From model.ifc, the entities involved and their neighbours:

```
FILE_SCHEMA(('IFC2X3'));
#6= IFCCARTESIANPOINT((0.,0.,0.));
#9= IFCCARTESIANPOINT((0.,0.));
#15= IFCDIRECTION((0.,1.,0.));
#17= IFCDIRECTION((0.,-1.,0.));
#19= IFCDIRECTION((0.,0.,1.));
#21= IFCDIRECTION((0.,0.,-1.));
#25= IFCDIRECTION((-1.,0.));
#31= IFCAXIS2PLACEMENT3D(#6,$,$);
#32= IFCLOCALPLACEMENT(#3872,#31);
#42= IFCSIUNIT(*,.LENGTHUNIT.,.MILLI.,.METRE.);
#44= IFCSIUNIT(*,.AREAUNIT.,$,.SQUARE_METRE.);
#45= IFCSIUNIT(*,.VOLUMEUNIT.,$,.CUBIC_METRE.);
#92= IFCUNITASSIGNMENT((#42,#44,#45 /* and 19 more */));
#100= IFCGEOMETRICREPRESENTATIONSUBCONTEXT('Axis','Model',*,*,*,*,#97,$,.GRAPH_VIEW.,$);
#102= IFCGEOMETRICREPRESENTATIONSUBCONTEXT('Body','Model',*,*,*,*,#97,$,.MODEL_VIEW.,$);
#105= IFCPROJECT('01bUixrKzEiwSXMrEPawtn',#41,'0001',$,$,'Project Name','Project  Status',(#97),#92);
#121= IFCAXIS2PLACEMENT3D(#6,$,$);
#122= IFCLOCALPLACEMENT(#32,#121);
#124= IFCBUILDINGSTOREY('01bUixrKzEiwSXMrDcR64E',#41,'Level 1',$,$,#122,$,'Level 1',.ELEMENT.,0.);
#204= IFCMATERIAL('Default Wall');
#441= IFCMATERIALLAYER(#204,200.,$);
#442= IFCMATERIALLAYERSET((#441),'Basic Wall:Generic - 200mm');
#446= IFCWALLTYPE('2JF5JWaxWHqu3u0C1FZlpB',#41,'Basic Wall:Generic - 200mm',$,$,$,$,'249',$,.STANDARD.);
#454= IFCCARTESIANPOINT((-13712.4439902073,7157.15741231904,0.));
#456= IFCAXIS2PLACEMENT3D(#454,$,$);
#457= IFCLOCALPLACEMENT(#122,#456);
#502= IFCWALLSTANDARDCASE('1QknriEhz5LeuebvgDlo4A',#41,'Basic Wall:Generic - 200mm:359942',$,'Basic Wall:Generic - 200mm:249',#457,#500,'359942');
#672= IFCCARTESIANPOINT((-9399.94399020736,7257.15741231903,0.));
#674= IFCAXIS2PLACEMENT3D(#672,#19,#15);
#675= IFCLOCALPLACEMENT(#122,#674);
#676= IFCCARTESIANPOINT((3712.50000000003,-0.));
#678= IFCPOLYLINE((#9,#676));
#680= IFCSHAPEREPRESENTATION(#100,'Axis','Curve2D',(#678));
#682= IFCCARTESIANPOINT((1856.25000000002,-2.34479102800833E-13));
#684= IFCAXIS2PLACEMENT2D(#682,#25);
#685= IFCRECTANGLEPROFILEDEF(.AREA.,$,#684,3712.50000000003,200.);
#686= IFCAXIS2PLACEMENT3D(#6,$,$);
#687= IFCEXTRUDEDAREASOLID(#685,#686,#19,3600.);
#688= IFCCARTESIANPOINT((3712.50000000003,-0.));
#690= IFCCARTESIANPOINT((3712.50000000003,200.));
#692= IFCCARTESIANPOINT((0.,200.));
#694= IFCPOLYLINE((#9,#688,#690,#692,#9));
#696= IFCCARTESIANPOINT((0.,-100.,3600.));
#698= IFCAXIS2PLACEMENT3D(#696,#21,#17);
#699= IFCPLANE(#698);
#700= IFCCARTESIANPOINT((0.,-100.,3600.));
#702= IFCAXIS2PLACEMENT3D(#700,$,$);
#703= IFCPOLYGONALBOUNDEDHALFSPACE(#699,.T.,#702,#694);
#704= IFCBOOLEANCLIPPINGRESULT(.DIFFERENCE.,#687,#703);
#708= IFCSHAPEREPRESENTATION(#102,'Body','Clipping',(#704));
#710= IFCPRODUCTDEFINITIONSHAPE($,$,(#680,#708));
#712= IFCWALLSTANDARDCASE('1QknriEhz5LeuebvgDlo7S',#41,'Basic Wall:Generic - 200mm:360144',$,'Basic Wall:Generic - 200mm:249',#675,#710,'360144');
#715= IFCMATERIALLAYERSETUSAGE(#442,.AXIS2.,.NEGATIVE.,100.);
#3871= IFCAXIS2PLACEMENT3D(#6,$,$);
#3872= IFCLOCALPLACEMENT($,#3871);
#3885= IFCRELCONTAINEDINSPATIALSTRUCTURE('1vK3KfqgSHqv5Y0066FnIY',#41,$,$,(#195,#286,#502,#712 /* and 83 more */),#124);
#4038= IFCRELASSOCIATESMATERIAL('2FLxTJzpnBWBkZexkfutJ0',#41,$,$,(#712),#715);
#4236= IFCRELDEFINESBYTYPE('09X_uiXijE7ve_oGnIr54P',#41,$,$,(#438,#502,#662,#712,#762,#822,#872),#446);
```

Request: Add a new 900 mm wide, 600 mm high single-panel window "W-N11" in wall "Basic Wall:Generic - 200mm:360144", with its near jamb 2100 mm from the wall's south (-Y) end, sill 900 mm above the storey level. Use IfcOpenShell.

```python
import numpy as np
import ifcopenshell
import ifcopenshell.api.feature
import ifcopenshell.api.geometry
import ifcopenshell.api.root
import ifcopenshell.api.spatial
import ifcopenshell.api.type
import ifcopenshell.geom
import ifcopenshell.util.element
import ifcopenshell.util.placement
import ifcopenshell.util.representation
import ifcopenshell.util.shape
import ifcopenshell.util.unit

model = ifcopenshell.open("model.ifc")
unit_scale = ifcopenshell.util.unit.calculate_unit_scale(model)
settings = ifcopenshell.geom.settings()


def volume(element):
    """Net volume in cubic metres, openings subtracted."""
    shape = ifcopenshell.geom.create_shape(settings, element)
    return ifcopenshell.util.shape.get_volume(shape.geometry)


wall = model.by_guid("1QknriEhz5LeuebvgDlo7S")
storey = ifcopenshell.util.element.get_container(wall, ifc_class="IfcBuildingStorey")
context = ifcopenshell.util.representation.get_context(model, "Model", "Body", "MODEL_VIEW")
before = volume(wall)

width, height, from_end, sill = 0.9, 0.6, 2.1, 0.9  # metres

# The wall runs along its own X axis, and the end named is its -X end.
wall_shape = ifcopenshell.geom.create_shape(settings, wall)
x, y, z = ifcopenshell.util.shape.get_vertices(wall_shape.geometry).T
start = x.min() + from_end
face, thickness = float(y.min()), float(y.max() - y.min())
wall_matrix = ifcopenshell.util.placement.get_local_placement(wall.ObjectPlacement)
level = ifcopenshell.util.placement.get_local_placement(storey.ObjectPlacement)[2, 3]


def in_wall(x, y):
    """Placement at x, y metres in the wall's axes, at sill height."""
    matrix = wall_matrix.copy()
    matrix[:, 3] = wall_matrix @ np.array([x / unit_scale, y / unit_scale, 0.0, 1.0])
    matrix[2, 3] = level + sill / unit_scale
    return matrix


# Opening: a box that overshoots both wall faces by 50 mm.
opening = ifcopenshell.api.root.create_entity(model, ifc_class="IfcOpeningElement")
box = ifcopenshell.api.geometry.add_wall_representation(
    model, context=context, length=width, height=height, thickness=thickness + 0.1
)
ifcopenshell.api.geometry.assign_representation(model, product=opening, representation=box)
ifcopenshell.api.geometry.edit_object_placement(model, product=opening, matrix=in_wall(start, face - 0.05), is_si=False)
ifcopenshell.api.feature.add_feature(model, feature=opening, element=wall)

window = ifcopenshell.api.root.create_entity(model, ifc_class="IfcWindow", name="W-N11")
window.OverallWidth, window.OverallHeight = width / unit_scale, height / unit_scale
body = ifcopenshell.api.geometry.add_window_representation(
    model,
    context=context,
    overall_width=window.OverallWidth,
    overall_height=window.OverallHeight,
    partition_type="SINGLE_PANEL",
)
ifcopenshell.api.geometry.assign_representation(model, product=window, representation=body)
ifcopenshell.api.spatial.assign_container(model, products=[window], relating_structure=storey)
fills = ifcopenshell.api.feature.add_filling(model, opening=opening, element=window)
fills.OwnerHistory = window.OwnerHistory  # required in IFC2X3

# IFC2X3 keeps the operation on the window style.
style = ifcopenshell.api.root.create_entity(model, ifc_class="IfcWindowStyle", name="W-N11")
style.OperationType, style.ConstructionType = "SINGLE_PANEL", "NOTDEFINED"
style.ParameterTakesPrecedence = style.Sizeable = False
ifcopenshell.api.type.assign_type(model, related_objects=[window], relating_type=style)

# Centre the window in the wall's thickness.
ifcopenshell.api.geometry.edit_object_placement(model, product=window, matrix=in_wall(start, face), is_si=False)
window_shape = ifcopenshell.geom.create_shape(settings, window)
depth = ifcopenshell.util.shape.get_vertices(window_shape.geometry)[:, 1]
offset = face + thickness / 2 - (depth.min() + depth.max()) / 2
ifcopenshell.api.geometry.edit_object_placement(model, product=window, matrix=in_wall(start, offset), is_si=False)

after = volume(wall)

print(f"wall volume {before:.3f} -> {after:.3f} m3")

model.write("model-out.ifc")
```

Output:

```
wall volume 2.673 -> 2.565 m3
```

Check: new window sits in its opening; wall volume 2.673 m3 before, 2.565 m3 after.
